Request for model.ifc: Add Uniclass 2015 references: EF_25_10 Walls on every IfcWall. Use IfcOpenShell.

First a look at what the model holds.

```python
import ifcopenshell

model = ifcopenshell.open("model.ifc")
print(model.schema)
print("classifications:", [c.Name for c in model.by_type("IfcClassification")])
for ifc_class in ("IfcDoor", "IfcRoof", "IfcStair", "IfcWall", "IfcWindow"):
    print(ifc_class, len(model.by_type(ifc_class)))
```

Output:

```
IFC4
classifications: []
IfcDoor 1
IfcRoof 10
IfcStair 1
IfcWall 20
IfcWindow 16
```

```python
import ifcopenshell
import ifcopenshell.api.classification

model = ifcopenshell.open("model.ifc")

system = ifcopenshell.api.classification.add_classification(model, classification="Uniclass 2015")

codes = {
    "IfcWall": ("EF_25_10", "Walls"),
}
for ifc_class, (code, name) in codes.items():
    products = model.by_type(ifc_class)
    ifcopenshell.api.classification.add_reference(
        model, products=products, classification=system, identification=code, name=name
    )
    print(code, len(products))

model.write("model-out.ifc")
```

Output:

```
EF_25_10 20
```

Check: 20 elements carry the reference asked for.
